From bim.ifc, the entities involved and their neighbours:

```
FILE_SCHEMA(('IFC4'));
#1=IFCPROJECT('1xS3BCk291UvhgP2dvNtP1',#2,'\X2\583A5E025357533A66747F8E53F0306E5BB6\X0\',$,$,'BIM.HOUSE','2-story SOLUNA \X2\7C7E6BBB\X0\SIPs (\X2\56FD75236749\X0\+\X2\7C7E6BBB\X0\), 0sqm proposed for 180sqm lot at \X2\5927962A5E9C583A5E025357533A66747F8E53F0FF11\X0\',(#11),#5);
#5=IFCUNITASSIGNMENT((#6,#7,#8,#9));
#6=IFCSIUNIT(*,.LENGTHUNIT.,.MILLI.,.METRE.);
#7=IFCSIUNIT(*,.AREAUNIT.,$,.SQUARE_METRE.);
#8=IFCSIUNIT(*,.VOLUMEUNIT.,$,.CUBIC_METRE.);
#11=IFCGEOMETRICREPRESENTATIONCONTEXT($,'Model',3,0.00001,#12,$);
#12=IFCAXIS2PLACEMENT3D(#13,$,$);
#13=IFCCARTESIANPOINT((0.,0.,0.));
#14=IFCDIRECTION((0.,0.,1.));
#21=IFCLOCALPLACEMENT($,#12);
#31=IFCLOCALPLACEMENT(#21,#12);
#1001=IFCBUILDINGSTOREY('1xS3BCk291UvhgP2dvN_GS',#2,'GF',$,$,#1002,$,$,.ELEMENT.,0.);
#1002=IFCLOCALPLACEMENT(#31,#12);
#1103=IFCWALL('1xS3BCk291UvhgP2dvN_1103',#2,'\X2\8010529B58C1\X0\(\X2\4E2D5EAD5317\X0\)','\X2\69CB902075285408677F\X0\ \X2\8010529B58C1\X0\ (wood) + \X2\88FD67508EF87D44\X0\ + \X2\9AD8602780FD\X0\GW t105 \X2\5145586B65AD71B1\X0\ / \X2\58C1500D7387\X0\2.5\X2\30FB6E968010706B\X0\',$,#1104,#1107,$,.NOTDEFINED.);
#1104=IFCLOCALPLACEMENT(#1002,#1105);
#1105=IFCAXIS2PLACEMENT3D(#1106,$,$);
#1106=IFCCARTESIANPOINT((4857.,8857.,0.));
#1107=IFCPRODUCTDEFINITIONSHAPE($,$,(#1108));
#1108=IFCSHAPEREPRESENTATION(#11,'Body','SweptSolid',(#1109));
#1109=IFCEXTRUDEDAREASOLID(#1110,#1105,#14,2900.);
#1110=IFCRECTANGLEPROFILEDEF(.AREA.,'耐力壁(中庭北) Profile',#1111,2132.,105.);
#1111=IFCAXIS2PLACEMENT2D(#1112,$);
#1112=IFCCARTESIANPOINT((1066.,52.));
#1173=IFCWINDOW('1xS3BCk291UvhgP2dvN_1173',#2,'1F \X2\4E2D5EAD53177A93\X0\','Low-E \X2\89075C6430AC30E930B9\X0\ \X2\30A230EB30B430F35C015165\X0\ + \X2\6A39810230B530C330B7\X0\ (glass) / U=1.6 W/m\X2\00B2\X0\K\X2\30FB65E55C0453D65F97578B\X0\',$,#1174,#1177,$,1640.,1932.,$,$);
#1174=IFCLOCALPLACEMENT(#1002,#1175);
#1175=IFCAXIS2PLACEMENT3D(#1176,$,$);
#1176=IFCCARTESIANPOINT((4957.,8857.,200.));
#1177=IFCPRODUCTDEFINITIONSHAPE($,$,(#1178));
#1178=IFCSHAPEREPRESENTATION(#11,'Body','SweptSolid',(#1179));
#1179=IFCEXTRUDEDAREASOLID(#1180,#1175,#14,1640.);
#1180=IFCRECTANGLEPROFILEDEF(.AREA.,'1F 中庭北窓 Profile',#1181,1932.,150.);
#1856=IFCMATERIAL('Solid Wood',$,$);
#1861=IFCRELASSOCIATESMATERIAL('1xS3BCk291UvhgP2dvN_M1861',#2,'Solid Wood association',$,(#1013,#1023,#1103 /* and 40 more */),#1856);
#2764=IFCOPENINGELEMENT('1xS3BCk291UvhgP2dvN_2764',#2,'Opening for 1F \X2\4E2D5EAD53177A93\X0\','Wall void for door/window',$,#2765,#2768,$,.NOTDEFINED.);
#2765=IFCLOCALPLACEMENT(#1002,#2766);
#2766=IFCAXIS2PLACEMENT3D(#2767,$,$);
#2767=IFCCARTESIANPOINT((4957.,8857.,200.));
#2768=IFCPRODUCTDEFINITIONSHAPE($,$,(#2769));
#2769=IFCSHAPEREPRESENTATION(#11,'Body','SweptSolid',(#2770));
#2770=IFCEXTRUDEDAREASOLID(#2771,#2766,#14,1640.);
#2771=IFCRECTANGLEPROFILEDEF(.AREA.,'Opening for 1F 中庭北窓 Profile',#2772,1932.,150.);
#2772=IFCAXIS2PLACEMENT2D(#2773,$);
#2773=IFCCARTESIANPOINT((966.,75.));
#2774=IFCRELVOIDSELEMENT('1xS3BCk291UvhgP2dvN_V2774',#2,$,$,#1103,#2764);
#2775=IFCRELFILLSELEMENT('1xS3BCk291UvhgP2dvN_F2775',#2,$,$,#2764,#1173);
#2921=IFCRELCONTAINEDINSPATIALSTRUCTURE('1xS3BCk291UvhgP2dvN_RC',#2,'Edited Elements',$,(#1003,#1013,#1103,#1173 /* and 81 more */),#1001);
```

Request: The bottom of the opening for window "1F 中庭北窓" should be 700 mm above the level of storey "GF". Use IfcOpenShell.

```python
import numpy as np
import ifcopenshell
import ifcopenshell.api.geometry
import ifcopenshell.geom
import ifcopenshell.util.element
import ifcopenshell.util.placement
import ifcopenshell.util.shape
import ifcopenshell.util.unit

model = ifcopenshell.open("bim.ifc")
unit_scale = ifcopenshell.util.unit.calculate_unit_scale(model)

window = model.by_id(1173)
opening = window.FillsVoids[0].RelatingOpeningElement
storey = ifcopenshell.util.element.get_container(window, ifc_class="IfcBuildingStorey")
level = ifcopenshell.util.placement.get_local_placement(storey.ObjectPlacement)[2, 3]

# The opening's origin need not be at the sill, so measure its lowest point.
shape = ifcopenshell.geom.create_shape(ifcopenshell.geom.settings(), opening)
bottom = ifcopenshell.util.shape.get_shape_bottom_elevation(shape, shape.geometry) / unit_scale
dz = level + 700.0 - bottom

shift = np.array([0.0, 0.0, dz])
# The window is not placed relative to its opening, so move both.
for product in (opening, window):
    matrix = ifcopenshell.util.placement.get_local_placement(product.ObjectPlacement)
    matrix[:3, 3] += shift
    ifcopenshell.api.geometry.edit_object_placement(model, product=product, matrix=matrix, is_si=False)

print(f"moved by {dz * unit_scale:+.3f} m")

model.write("bim_v2.ifc")
```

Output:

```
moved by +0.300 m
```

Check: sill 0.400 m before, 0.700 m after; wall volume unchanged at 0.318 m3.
